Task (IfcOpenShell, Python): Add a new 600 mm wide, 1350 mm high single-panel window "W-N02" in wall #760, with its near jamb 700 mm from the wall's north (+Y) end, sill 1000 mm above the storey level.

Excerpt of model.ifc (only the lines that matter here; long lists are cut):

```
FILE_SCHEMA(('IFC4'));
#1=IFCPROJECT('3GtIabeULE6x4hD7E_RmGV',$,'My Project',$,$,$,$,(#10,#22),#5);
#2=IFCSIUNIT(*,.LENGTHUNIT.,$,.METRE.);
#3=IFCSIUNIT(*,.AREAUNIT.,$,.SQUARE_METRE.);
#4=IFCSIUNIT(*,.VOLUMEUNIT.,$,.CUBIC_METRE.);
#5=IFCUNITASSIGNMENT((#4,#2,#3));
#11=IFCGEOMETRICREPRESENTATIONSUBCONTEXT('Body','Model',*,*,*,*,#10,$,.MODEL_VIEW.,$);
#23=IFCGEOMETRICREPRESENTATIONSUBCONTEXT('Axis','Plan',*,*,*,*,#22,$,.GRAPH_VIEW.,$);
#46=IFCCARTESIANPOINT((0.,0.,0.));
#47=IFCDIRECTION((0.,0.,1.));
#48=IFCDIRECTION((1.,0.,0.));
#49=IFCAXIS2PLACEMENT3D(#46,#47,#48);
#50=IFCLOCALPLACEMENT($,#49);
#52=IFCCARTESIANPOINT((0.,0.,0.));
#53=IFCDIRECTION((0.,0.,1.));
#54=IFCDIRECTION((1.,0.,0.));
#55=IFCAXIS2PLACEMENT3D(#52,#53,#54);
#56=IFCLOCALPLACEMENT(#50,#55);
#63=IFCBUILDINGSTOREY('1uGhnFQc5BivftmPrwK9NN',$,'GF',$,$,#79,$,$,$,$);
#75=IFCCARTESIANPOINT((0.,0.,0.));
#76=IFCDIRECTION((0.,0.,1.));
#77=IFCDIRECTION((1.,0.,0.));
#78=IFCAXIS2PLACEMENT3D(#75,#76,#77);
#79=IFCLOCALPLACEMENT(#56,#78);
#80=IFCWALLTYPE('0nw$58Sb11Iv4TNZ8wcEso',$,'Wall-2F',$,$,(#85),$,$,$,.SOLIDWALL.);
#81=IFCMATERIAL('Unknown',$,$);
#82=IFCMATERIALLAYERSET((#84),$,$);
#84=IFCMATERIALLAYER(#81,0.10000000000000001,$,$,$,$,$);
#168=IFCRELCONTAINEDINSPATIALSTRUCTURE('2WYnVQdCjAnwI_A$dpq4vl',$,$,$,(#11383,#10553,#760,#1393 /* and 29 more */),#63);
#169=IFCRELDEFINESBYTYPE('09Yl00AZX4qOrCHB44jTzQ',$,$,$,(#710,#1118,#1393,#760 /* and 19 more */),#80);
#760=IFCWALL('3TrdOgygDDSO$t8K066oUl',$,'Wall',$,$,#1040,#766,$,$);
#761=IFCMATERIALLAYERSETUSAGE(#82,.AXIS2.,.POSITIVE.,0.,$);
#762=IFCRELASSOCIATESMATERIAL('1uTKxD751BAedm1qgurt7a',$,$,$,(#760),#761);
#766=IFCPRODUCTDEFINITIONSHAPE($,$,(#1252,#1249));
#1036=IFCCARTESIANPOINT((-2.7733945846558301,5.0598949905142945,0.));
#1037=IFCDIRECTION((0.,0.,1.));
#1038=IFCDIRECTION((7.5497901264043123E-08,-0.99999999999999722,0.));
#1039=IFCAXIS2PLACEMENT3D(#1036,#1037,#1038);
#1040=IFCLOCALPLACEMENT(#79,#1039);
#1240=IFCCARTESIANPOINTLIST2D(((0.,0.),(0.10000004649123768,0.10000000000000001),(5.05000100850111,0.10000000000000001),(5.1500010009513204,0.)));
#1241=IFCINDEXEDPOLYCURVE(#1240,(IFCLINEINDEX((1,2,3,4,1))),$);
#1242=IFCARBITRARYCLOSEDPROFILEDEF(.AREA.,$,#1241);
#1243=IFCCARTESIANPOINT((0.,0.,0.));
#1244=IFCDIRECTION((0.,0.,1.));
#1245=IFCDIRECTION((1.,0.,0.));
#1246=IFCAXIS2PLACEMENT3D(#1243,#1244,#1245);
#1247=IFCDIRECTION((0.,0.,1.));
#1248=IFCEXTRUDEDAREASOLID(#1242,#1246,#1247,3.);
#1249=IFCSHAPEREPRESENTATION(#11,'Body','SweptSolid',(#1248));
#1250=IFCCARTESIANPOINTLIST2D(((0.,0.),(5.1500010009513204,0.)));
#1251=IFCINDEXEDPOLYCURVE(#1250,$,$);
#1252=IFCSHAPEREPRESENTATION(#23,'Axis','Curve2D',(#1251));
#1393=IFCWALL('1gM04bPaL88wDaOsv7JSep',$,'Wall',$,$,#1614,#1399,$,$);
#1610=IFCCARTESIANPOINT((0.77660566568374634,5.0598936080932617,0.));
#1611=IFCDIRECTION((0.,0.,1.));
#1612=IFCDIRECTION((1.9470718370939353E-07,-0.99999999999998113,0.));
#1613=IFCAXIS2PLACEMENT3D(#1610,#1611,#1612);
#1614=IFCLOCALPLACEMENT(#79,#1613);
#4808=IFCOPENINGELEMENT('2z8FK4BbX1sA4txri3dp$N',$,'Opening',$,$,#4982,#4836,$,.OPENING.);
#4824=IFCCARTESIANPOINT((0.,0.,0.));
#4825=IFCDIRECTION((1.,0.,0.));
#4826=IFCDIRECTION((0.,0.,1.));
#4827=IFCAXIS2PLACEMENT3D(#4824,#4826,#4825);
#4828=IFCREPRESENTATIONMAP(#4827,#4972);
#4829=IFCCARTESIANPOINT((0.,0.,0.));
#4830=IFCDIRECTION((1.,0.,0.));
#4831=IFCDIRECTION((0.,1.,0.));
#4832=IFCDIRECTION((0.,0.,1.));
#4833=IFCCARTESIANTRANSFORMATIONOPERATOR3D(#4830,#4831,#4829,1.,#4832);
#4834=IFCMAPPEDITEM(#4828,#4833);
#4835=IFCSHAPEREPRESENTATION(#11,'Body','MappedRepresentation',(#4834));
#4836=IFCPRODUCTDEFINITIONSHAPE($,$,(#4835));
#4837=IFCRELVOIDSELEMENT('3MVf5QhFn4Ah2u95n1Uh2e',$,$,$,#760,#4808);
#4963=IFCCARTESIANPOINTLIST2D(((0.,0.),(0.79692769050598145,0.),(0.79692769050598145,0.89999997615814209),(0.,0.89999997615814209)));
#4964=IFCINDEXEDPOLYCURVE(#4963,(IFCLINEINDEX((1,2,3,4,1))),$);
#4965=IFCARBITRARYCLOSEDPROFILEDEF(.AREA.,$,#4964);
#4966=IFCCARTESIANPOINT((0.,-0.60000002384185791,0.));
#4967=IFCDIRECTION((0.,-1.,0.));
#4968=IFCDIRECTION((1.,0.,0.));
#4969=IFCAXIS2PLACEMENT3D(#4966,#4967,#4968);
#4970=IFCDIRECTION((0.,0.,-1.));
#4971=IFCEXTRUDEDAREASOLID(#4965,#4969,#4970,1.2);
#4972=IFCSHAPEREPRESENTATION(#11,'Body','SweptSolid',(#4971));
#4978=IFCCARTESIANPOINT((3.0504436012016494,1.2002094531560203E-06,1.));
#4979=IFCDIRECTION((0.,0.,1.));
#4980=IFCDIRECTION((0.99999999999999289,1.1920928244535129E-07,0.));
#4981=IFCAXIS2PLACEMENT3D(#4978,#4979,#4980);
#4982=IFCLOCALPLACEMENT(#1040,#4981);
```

```python
import numpy as np
import ifcopenshell
import ifcopenshell.api.feature
import ifcopenshell.api.geometry
import ifcopenshell.api.root
import ifcopenshell.api.spatial
import ifcopenshell.geom
import ifcopenshell.util.element
import ifcopenshell.util.placement
import ifcopenshell.util.representation
import ifcopenshell.util.shape
import ifcopenshell.util.unit

model = ifcopenshell.open("model.ifc")
unit_scale = ifcopenshell.util.unit.calculate_unit_scale(model)
settings = ifcopenshell.geom.settings()


def volume(element):
    """Net volume in cubic metres, openings subtracted."""
    shape = ifcopenshell.geom.create_shape(settings, element)
    return ifcopenshell.util.shape.get_volume(shape.geometry)


wall = model.by_guid("3TrdOgygDDSO$t8K066oUl")
storey = ifcopenshell.util.element.get_container(wall, ifc_class="IfcBuildingStorey")
context = ifcopenshell.util.representation.get_context(model, "Model", "Body", "MODEL_VIEW")
before = volume(wall)

width, height, from_end, sill = 0.6, 1.35, 0.7, 1  # metres

# The wall runs along its own X axis, and the end named is its -X end.
wall_shape = ifcopenshell.geom.create_shape(settings, wall)
x, y, z = ifcopenshell.util.shape.get_vertices(wall_shape.geometry).T
start = x.min() + from_end
face, thickness = float(y.min()), float(y.max() - y.min())
wall_matrix = ifcopenshell.util.placement.get_local_placement(wall.ObjectPlacement)
level = ifcopenshell.util.placement.get_local_placement(storey.ObjectPlacement)[2, 3]


def in_wall(x, y):
    """Placement at x, y metres in the wall's axes, at sill height."""
    matrix = wall_matrix.copy()
    matrix[:, 3] = wall_matrix @ np.array([x / unit_scale, y / unit_scale, 0.0, 1.0])
    matrix[2, 3] = level + sill / unit_scale
    return matrix


# Opening: a box that overshoots both wall faces by 50 mm.
opening = ifcopenshell.api.root.create_entity(model, ifc_class="IfcOpeningElement", predefined_type="OPENING")
box = ifcopenshell.api.geometry.add_wall_representation(
    model, context=context, length=width, height=height, thickness=thickness + 0.1
)
ifcopenshell.api.geometry.assign_representation(model, product=opening, representation=box)
ifcopenshell.api.geometry.edit_object_placement(model, product=opening, matrix=in_wall(start, face - 0.05), is_si=False)
ifcopenshell.api.feature.add_feature(model, feature=opening, element=wall)

window = ifcopenshell.api.root.create_entity(model, ifc_class="IfcWindow", name="W-N02", predefined_type="WINDOW")
window.OverallWidth, window.OverallHeight = width / unit_scale, height / unit_scale
window.PartitioningType = "SINGLE_PANEL"
body = ifcopenshell.api.geometry.add_window_representation(
    model,
    context=context,
    overall_width=window.OverallWidth,
    overall_height=window.OverallHeight,
    partition_type="SINGLE_PANEL",
)
ifcopenshell.api.geometry.assign_representation(model, product=window, representation=body)
ifcopenshell.api.spatial.assign_container(model, products=[window], relating_structure=storey)
ifcopenshell.api.feature.add_filling(model, opening=opening, element=window)

# Centre the window in the wall's thickness.
ifcopenshell.api.geometry.edit_object_placement(model, product=window, matrix=in_wall(start, face), is_si=False)
window_shape = ifcopenshell.geom.create_shape(settings, window)
depth = ifcopenshell.util.shape.get_vertices(window_shape.geometry)[:, 1]
offset = face + thickness / 2 - (depth.min() + depth.max()) / 2
ifcopenshell.api.geometry.edit_object_placement(model, product=window, matrix=in_wall(start, offset), is_si=False)

after = volume(wall)

print(f"wall volume {before:.3f} -> {after:.3f} m3")

model.write("model-out.ifc")
```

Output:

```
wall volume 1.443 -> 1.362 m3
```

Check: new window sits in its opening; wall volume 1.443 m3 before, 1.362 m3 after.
